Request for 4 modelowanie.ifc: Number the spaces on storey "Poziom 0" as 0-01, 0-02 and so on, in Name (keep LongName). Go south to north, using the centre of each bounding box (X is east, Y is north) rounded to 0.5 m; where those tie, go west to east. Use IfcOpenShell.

First a look at what the model holds.

```python
import ifcopenshell
import ifcopenshell.util.element
import ifcopenshell.util.placement

model = ifcopenshell.open("4 modelowanie.ifc")
print(model.schema)
storey = next(s for s in model.by_type("IfcBuildingStorey") if s.Name == "Poziom 0")
spaces = [e for e in ifcopenshell.util.element.get_decomposition(storey) if e.is_a("IfcSpace")]
for e in sorted(spaces, key=lambda e: e.id()):
    origin = ifcopenshell.util.placement.get_local_placement(e.ObjectPlacement)[:3, 3]
    print(e.id(), e.Name, e.LongName, origin.round(2) + 0.0, sep=" | ")
```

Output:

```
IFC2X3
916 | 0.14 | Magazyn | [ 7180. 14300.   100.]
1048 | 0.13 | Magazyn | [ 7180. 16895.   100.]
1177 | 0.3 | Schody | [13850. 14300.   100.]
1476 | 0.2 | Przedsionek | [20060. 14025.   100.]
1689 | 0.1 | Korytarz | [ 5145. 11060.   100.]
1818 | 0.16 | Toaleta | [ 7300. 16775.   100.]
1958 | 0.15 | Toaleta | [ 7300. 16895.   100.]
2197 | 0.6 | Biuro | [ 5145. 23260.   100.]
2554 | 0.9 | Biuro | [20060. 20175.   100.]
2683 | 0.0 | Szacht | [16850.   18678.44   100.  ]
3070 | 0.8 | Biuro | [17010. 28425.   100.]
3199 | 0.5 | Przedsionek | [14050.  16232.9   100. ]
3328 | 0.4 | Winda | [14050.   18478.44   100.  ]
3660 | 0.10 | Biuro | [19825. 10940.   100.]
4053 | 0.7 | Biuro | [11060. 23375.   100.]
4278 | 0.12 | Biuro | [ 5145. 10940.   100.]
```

```python
import ifcopenshell
import ifcopenshell.geom
import ifcopenshell.util.element
import ifcopenshell.util.shape

model = ifcopenshell.open("4 modelowanie.ifc")
settings = ifcopenshell.geom.settings()
settings.set("use-world-coords", True)


def centre(element):
    shape = ifcopenshell.geom.create_shape(settings, element)
    return ifcopenshell.util.shape.get_bbox_centroid(shape.geometry)


storey = next(s for s in model.by_type("IfcBuildingStorey") if s.Name == "Poziom 0")
spaces = [e for e in ifcopenshell.util.element.get_decomposition(storey) if e.is_a("IfcSpace")]

# Insertion points can sit at a corner or the storey origin, so sort by the geometry (in metres).
centres = {e: centre(e) for e in spaces}
spaces.sort(key=lambda e: (round(centres[e][1] / 0.5), centres[e][0]))

for i, e in enumerate(spaces, start=1):
    number = f"0-{i:02d}"
    e.Name = number
    print(e.id(), number)

model.write("4 modelowanie-out.ifc")
```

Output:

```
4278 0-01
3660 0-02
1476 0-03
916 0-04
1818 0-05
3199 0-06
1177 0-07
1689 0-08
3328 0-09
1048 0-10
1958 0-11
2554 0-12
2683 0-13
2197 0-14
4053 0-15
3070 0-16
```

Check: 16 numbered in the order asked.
